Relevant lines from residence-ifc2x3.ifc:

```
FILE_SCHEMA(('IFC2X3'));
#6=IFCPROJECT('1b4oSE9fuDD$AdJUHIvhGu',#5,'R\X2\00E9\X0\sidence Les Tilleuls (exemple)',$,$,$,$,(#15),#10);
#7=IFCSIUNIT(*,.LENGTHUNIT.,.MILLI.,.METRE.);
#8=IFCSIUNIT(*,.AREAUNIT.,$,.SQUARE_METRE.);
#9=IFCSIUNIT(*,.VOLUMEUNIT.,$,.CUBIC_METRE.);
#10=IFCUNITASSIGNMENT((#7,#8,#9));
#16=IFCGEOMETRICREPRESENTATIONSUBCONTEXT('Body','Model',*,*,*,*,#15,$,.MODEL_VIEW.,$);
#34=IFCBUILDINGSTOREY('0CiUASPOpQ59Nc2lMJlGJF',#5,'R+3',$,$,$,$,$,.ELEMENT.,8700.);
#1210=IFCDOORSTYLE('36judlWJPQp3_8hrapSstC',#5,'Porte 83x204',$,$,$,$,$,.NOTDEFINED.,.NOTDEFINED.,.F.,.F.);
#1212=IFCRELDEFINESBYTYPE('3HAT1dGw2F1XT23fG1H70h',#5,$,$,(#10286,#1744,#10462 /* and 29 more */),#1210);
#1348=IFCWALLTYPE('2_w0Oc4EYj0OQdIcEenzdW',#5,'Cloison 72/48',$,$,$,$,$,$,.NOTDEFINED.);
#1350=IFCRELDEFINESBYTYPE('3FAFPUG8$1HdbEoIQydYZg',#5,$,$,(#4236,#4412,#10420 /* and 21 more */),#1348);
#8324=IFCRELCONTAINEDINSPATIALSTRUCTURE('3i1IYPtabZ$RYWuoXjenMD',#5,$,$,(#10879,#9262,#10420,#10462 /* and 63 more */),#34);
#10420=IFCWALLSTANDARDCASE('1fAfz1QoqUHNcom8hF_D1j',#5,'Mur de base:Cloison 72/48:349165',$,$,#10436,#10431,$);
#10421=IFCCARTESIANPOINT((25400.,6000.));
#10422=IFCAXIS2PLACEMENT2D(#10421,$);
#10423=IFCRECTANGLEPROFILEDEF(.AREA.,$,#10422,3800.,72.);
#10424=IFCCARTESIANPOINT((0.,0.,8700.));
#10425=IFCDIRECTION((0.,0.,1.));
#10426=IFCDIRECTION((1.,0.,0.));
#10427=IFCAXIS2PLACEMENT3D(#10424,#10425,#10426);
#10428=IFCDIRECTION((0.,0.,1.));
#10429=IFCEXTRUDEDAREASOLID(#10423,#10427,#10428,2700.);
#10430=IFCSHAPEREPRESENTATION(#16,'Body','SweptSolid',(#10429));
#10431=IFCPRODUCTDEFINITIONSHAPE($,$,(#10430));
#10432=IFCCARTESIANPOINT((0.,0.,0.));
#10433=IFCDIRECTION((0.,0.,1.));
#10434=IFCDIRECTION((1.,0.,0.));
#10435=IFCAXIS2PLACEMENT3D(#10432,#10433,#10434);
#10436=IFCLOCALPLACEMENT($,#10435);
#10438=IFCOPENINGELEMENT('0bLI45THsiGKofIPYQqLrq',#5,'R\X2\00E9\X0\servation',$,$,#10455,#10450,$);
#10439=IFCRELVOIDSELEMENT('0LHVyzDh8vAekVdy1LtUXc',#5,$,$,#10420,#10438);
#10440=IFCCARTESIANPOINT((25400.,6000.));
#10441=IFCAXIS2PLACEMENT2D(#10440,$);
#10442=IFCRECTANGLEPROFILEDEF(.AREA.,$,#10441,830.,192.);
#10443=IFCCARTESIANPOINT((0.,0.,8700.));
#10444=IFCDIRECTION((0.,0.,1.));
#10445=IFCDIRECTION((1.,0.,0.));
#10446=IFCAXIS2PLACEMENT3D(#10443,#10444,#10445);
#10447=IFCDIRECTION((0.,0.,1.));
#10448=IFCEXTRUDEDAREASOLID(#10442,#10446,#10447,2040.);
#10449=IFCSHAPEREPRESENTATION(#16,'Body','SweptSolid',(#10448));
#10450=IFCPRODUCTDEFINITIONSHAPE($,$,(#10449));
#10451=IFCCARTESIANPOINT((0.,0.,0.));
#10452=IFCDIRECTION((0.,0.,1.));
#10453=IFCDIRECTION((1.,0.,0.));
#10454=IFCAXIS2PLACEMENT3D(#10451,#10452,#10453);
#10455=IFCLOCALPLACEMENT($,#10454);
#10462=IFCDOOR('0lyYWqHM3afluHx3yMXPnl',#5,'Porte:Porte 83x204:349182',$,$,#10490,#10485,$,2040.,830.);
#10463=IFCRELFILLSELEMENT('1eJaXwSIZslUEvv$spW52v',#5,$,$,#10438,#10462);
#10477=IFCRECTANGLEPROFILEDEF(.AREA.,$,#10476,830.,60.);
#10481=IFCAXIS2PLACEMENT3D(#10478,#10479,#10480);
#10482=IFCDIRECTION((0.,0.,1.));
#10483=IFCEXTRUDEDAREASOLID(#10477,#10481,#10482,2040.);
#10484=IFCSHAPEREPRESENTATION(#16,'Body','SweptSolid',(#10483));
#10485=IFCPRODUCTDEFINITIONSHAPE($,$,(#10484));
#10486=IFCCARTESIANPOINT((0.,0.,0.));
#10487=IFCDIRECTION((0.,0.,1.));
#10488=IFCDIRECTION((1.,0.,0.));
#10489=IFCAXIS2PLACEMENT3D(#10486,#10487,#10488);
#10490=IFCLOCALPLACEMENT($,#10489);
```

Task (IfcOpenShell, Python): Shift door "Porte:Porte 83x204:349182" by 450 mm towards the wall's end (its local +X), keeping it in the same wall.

```python
import ifcopenshell
import ifcopenshell.api.geometry
import ifcopenshell.util.placement
import ifcopenshell.util.unit

model = ifcopenshell.open("residence-ifc2x3.ifc")
unit_scale = ifcopenshell.util.unit.calculate_unit_scale(model)

door = model.by_guid("0lyYWqHM3afluHx3yMXPnl")
opening = door.FillsVoids[0].RelatingOpeningElement
wall = opening.VoidsElements[0].RelatingBuildingElement

wall_matrix = ifcopenshell.util.placement.get_local_placement(wall.ObjectPlacement)
shift = wall_matrix[:3, 0] * 0.45 / unit_scale
before = ifcopenshell.util.placement.get_local_placement(door.ObjectPlacement)[:3, 3].copy()

# The door is not placed relative to its opening, so move both.
for product in (opening, door):
    matrix = ifcopenshell.util.placement.get_local_placement(product.ObjectPlacement)
    matrix[:3, 3] += shift
    ifcopenshell.api.geometry.edit_object_placement(model, product=product, matrix=matrix, is_si=False)

after = ifcopenshell.util.placement.get_local_placement(door.ObjectPlacement)[:3, 3]
print("door moved by", (after - before).round(3) + 0.0)

model.write("residence-ifc2x3_v2.ifc")
```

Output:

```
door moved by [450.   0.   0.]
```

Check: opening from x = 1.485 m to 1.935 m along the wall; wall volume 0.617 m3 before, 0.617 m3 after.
